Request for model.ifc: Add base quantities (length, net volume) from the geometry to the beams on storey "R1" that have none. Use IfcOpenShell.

First a look at what the model holds.

```python
import ifcopenshell
import ifcopenshell.util.element
import ifcopenshell.util.unit

model = ifcopenshell.open("model.ifc")
print(model.schema)
for unit_type in ("LENGTHUNIT", "AREAUNIT", "VOLUMEUNIT"):
    print(unit_type, ifcopenshell.util.unit.calculate_unit_scale(model, unit_type))
storey = next(s for s in model.by_type("IfcBuildingStorey") if s.Name == "R1")
beams = [e for e in ifcopenshell.util.element.get_decomposition(storey) if e.is_a("IfcBeam")]
for e in sorted(beams, key=lambda e: e.id()):
    print(e.id(), e.is_a(), e.Name, list(ifcopenshell.util.element.get_psets(e, qtos_only=True)), sep=" | ")
```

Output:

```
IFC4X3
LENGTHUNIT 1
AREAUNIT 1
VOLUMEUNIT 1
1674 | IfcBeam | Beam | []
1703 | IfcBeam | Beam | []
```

```python
import ifcopenshell
import ifcopenshell.api.pset
import ifcopenshell.geom
import ifcopenshell.util.element
import ifcopenshell.util.shape
import ifcopenshell.util.unit

model = ifcopenshell.open("model.ifc")
unit_scale = ifcopenshell.util.unit.calculate_unit_scale(model)
volume_scale = ifcopenshell.util.unit.calculate_unit_scale(model, "VOLUMEUNIT")
settings = ifcopenshell.geom.settings()

storey = next(s for s in model.by_type("IfcBuildingStorey") if s.Name == "R1")
beams = [e for e in ifcopenshell.util.element.get_decomposition(storey) if e.is_a("IfcBeam")]

for e in sorted(beams, key=lambda e: e.id()):
    if ifcopenshell.util.element.get_psets(e, qtos_only=True, should_inherit=False):
        continue
    # Geometry comes back in metres, in the element's own axes.
    shape = ifcopenshell.geom.create_shape(settings, e)
    values = {
        "Length": ifcopenshell.util.shape.get_max_xyz(shape.geometry) / unit_scale,
        "NetVolume": ifcopenshell.util.shape.get_volume(shape.geometry) / volume_scale,
    }
    qto = ifcopenshell.api.pset.add_qto(model, product=e, name="Qto_BeamBaseQuantities")
    ifcopenshell.api.pset.edit_qto(model, qto=qto, properties=values)
    print(e.id(), {k: round(v, 3) for k, v in values.items()})

model.write("model_rev.ifc")
```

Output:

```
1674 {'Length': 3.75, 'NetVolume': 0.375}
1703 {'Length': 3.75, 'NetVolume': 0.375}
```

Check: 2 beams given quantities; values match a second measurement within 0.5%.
